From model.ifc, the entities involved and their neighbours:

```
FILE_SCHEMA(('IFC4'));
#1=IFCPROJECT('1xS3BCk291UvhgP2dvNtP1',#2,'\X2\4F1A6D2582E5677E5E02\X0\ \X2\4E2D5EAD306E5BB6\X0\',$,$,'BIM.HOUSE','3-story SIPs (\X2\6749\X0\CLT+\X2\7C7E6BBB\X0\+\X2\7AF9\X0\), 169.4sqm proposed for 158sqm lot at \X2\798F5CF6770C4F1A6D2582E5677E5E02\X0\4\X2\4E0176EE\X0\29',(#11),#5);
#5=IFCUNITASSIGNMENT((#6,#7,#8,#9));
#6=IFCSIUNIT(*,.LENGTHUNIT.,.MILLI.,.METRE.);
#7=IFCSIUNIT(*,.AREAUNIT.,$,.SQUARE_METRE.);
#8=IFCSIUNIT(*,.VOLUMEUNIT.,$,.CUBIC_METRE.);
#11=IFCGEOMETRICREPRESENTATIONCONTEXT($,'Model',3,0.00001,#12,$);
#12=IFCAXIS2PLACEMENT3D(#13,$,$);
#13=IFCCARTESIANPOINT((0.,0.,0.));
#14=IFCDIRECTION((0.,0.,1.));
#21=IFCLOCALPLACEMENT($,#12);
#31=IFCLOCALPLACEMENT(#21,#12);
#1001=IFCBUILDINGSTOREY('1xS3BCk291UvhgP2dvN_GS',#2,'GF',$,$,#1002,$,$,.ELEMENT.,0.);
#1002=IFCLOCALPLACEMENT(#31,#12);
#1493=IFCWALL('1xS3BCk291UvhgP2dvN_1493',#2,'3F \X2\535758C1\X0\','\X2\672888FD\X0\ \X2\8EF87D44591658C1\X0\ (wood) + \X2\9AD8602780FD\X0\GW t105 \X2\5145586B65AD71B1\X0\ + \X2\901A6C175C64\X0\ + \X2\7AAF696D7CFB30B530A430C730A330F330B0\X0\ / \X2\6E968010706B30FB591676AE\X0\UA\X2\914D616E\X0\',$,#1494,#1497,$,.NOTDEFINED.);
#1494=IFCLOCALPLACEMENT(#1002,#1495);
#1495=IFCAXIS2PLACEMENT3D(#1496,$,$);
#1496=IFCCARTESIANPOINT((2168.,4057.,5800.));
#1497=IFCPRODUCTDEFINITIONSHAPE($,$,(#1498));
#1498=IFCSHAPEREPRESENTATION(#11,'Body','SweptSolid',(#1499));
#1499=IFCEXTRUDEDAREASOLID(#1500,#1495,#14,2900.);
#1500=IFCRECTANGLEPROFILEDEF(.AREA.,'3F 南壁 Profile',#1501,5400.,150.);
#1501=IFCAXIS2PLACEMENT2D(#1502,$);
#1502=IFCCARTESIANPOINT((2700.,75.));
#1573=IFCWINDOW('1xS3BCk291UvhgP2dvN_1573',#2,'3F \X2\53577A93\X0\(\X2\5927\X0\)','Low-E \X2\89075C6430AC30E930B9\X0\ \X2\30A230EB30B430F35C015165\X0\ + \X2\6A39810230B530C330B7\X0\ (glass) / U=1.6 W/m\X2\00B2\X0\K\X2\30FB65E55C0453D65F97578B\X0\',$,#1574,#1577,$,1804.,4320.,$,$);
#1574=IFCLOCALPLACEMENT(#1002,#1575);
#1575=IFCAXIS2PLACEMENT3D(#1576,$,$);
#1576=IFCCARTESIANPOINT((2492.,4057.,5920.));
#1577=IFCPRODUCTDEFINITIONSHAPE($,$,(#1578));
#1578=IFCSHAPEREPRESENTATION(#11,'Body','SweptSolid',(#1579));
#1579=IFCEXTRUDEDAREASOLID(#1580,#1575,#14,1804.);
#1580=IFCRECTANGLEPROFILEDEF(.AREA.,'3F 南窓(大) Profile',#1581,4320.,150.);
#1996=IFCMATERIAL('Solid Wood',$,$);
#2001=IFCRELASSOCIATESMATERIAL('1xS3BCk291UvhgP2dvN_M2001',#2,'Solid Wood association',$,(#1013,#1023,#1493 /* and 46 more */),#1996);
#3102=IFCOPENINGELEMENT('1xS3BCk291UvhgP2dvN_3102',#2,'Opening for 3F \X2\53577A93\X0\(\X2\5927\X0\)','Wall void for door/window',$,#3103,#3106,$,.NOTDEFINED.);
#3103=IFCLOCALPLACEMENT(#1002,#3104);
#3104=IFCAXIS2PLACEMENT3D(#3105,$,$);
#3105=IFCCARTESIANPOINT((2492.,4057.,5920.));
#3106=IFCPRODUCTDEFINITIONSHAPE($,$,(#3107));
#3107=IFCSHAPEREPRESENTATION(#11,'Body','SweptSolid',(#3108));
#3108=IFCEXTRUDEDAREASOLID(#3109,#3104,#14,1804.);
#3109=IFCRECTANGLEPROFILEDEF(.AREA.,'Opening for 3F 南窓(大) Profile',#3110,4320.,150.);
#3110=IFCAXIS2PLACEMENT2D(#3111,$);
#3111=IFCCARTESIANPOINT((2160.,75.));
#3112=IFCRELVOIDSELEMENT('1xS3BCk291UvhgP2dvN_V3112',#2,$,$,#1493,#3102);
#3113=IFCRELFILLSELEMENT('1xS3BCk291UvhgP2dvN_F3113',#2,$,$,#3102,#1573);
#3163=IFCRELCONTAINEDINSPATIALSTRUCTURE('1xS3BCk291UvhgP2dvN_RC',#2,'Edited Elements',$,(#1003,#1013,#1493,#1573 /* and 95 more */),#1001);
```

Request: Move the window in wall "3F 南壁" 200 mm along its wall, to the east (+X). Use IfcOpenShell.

```python
import ifcopenshell
import ifcopenshell.api.geometry
import ifcopenshell.util.placement
import ifcopenshell.util.unit

model = ifcopenshell.open("model.ifc")
unit_scale = ifcopenshell.util.unit.calculate_unit_scale(model)

window = model.by_guid("1xS3BCk291UvhgP2dvN_1573")
opening = window.FillsVoids[0].RelatingOpeningElement
wall = opening.VoidsElements[0].RelatingBuildingElement

wall_matrix = ifcopenshell.util.placement.get_local_placement(wall.ObjectPlacement)
shift = wall_matrix[:3, 0] * 0.2 / unit_scale
before = ifcopenshell.util.placement.get_local_placement(window.ObjectPlacement)[:3, 3].copy()

# The window is not placed relative to its opening, so move both.
for product in (opening, window):
    matrix = ifcopenshell.util.placement.get_local_placement(product.ObjectPlacement)
    matrix[:3, 3] += shift
    ifcopenshell.api.geometry.edit_object_placement(model, product=product, matrix=matrix, is_si=False)

after = ifcopenshell.util.placement.get_local_placement(window.ObjectPlacement)[:3, 3]
print("window moved by", (after - before).round(3) + 0.0)

model.write("model_v2.ifc")
```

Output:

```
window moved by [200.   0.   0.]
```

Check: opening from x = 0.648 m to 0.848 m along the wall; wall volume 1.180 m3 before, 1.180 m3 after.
